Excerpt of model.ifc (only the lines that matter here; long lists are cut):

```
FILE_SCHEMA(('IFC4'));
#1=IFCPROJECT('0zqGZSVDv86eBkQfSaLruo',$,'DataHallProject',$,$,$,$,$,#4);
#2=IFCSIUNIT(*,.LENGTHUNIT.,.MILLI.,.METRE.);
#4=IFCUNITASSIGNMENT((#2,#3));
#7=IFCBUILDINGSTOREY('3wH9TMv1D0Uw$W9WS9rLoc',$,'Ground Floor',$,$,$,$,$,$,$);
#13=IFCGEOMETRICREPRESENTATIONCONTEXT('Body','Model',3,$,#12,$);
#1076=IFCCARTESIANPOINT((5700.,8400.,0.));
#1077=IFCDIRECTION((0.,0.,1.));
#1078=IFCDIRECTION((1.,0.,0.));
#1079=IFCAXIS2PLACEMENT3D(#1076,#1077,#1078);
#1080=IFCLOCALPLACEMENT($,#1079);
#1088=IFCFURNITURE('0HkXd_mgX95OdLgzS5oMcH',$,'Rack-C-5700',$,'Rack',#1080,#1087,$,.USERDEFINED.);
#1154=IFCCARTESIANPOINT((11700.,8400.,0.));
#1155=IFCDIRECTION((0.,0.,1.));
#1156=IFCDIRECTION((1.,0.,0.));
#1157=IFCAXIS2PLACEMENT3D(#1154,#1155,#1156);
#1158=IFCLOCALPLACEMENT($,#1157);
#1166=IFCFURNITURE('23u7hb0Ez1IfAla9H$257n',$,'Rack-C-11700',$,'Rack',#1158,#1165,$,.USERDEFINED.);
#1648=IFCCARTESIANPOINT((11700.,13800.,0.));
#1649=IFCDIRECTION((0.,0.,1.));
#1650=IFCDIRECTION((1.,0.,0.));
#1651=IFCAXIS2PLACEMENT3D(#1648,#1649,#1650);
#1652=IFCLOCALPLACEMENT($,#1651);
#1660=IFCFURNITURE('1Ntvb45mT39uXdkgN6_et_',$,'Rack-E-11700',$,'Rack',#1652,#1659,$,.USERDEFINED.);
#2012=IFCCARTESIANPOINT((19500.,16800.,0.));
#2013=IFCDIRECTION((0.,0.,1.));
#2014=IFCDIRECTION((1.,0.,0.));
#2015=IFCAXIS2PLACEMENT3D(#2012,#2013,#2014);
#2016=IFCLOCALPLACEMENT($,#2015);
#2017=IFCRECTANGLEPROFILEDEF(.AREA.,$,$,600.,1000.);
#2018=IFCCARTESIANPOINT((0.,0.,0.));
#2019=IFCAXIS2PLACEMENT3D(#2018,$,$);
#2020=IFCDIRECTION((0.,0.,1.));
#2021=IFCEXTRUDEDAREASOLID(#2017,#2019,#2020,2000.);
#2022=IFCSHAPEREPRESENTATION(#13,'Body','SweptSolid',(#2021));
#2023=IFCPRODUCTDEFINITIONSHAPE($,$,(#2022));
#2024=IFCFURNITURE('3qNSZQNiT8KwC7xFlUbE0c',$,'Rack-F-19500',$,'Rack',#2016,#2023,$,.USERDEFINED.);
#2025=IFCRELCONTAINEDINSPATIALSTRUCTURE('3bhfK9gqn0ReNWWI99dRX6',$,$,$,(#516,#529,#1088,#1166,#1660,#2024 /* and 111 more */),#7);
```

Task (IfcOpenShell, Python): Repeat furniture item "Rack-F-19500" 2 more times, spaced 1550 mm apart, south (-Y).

```python
import numpy as np
import ifcopenshell
import ifcopenshell.api.geometry
import ifcopenshell.api.root
import ifcopenshell.util.element
import ifcopenshell.util.placement
import ifcopenshell.util.unit

model = ifcopenshell.open("model.ifc")
unit_scale = ifcopenshell.util.unit.calculate_unit_scale(model)

source = model.by_guid("3qNSZQNiT8KwC7xFlUbE0c")
base = ifcopenshell.util.placement.get_local_placement(source.ObjectPlacement)
step = np.array([0.0, -1.0, 0.0]) * 1.55 / unit_scale

for i in range(1, 3):
    copy = ifcopenshell.api.root.copy_class(model, product=source)
    copy.Representation = ifcopenshell.util.element.copy_deep(
        model, source.Representation, exclude=["IfcGeometricRepresentationContext", "IfcRepresentationMap"]
    )
    matrix = base.copy()
    matrix[:3, 3] += i * step
    print("added at", matrix[:3, 3].round(3) + 0.0)
    ifcopenshell.api.geometry.edit_object_placement(model, product=copy, matrix=matrix, is_si=False)

model.write("model_v2.ifc")
```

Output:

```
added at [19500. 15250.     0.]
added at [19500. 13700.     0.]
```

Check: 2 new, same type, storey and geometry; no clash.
